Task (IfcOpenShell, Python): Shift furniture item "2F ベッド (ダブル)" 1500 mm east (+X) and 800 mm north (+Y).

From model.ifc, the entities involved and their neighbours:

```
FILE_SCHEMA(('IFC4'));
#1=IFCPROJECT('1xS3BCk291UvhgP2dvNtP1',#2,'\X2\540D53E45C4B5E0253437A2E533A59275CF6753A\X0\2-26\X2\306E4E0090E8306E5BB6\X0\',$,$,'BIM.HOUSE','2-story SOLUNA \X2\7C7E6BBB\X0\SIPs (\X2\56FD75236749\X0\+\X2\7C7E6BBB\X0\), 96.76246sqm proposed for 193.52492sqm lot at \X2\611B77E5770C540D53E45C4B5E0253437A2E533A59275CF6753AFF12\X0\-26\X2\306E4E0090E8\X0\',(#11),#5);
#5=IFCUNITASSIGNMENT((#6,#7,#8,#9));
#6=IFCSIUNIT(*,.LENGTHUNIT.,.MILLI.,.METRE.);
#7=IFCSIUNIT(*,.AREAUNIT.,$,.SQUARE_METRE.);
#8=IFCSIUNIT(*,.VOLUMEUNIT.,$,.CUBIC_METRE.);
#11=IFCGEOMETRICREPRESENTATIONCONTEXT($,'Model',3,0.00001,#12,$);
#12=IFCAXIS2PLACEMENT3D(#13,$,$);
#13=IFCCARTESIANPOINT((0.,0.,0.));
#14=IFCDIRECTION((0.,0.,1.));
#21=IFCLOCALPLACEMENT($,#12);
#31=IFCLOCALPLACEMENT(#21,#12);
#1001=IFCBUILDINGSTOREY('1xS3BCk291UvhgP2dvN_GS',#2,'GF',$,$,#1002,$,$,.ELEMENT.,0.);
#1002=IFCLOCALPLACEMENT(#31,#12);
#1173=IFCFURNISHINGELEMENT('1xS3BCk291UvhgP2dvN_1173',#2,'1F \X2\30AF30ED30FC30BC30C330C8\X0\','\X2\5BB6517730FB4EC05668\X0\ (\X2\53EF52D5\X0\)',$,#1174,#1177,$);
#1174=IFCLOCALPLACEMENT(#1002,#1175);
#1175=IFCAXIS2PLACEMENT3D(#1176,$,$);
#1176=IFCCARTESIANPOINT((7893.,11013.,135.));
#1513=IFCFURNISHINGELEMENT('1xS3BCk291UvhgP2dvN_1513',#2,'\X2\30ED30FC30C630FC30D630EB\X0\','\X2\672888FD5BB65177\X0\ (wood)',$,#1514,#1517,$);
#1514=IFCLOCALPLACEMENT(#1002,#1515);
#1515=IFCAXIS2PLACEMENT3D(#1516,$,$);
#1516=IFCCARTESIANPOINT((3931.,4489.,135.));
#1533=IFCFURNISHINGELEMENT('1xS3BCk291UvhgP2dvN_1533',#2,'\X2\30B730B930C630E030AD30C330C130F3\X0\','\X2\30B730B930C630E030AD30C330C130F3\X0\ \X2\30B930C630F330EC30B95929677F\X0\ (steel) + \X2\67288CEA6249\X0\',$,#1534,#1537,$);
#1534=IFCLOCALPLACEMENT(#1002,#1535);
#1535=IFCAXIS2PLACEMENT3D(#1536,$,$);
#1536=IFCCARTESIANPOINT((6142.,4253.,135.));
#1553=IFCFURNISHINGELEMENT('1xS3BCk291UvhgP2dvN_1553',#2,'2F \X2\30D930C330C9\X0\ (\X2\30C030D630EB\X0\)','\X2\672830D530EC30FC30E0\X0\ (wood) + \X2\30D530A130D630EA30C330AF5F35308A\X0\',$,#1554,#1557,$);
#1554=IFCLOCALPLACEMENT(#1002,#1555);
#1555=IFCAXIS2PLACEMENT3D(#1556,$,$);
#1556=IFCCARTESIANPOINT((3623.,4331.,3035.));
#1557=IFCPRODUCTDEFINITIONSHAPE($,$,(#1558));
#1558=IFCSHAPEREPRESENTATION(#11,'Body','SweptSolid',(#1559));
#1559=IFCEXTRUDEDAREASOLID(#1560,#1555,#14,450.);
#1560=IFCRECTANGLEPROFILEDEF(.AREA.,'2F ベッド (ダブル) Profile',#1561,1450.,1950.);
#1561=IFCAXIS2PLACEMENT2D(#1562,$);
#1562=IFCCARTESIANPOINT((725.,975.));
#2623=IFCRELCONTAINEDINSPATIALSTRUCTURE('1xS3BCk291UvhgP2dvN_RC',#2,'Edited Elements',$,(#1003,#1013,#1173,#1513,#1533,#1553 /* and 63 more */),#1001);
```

```python
import ifcopenshell
import ifcopenshell.api.geometry
import ifcopenshell.util.placement
import ifcopenshell.util.unit

model = ifcopenshell.open("model.ifc")
unit_scale = ifcopenshell.util.unit.calculate_unit_scale(model)

item = model.by_id(1553)
matrix = ifcopenshell.util.placement.get_local_placement(item.ObjectPlacement)
matrix[0, 3] += 1.5 / unit_scale
matrix[1, 3] += 0.8 / unit_scale
ifcopenshell.api.geometry.edit_object_placement(model, product=item, matrix=matrix, is_si=False)

print(ifcopenshell.util.placement.get_local_placement(item.ObjectPlacement).round(3) + 0.0)

model.write("model_rev.ifc")
```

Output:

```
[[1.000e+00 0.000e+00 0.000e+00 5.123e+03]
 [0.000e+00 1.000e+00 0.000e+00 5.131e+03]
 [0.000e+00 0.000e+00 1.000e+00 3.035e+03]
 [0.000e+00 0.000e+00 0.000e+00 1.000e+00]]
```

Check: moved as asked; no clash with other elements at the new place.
